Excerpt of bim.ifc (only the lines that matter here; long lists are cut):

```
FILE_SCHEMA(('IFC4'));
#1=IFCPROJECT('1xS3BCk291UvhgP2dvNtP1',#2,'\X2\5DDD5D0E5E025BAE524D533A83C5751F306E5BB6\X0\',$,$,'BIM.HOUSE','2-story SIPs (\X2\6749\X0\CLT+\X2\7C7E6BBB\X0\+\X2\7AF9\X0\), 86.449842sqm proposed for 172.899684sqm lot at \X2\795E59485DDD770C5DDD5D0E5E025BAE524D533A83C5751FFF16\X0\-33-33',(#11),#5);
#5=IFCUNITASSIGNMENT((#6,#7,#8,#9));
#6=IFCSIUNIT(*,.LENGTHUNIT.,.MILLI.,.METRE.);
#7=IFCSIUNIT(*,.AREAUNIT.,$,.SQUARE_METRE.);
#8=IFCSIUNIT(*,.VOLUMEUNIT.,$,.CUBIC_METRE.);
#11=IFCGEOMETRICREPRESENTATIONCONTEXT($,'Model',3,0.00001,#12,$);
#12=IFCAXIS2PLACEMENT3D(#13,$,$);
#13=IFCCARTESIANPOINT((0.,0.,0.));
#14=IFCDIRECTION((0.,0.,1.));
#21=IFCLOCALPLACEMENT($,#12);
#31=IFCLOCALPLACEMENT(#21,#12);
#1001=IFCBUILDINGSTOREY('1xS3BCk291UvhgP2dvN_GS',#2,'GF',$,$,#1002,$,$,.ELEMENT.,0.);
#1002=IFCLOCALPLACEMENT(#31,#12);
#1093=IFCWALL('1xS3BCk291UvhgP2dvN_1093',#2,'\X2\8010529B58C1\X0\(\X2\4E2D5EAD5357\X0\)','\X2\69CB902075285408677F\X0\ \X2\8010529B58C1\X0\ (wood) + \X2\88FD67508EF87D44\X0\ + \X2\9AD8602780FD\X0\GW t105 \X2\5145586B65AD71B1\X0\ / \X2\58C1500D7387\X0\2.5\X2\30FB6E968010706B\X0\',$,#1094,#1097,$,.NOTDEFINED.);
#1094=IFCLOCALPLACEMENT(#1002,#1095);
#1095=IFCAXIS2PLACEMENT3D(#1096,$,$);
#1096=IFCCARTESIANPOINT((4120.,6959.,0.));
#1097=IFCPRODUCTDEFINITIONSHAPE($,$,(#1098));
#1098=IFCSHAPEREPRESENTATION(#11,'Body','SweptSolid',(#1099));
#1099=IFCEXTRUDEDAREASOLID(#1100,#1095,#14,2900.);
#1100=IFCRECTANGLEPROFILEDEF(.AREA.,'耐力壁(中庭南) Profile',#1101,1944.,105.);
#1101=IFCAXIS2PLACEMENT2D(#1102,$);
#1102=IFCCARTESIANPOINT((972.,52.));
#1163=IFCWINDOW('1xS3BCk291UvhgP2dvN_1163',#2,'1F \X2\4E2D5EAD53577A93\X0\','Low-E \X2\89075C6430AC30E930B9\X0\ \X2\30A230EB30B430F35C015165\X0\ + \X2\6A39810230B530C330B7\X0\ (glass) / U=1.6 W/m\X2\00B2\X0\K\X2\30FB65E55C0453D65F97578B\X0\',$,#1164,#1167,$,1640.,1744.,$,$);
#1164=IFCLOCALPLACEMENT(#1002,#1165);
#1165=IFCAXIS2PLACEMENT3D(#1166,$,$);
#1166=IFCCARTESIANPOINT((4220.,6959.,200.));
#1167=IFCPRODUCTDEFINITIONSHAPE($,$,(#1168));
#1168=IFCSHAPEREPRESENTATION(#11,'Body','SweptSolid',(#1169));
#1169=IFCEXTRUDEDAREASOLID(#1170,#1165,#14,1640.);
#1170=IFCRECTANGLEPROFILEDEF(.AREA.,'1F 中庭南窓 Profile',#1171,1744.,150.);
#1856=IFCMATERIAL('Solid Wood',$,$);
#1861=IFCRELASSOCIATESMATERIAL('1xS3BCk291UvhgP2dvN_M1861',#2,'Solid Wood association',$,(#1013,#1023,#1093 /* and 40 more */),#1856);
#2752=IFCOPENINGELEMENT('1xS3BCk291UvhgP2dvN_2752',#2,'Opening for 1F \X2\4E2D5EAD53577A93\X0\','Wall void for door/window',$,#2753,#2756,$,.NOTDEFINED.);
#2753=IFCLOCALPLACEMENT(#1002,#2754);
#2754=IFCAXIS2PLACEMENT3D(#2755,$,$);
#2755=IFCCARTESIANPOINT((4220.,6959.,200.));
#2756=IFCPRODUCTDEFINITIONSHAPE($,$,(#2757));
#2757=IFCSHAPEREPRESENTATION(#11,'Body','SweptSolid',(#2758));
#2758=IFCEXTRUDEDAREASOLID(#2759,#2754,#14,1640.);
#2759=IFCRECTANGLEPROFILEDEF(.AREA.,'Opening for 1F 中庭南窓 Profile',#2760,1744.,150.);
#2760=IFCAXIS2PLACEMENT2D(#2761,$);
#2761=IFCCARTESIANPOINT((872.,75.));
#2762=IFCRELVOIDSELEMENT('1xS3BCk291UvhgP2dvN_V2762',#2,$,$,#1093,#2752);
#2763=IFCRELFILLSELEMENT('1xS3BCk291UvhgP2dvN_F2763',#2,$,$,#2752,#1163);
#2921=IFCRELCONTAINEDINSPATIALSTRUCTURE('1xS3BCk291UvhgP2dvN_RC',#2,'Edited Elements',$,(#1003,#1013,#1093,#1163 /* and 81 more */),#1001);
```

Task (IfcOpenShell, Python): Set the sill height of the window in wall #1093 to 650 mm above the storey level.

```python
import numpy as np
import ifcopenshell
import ifcopenshell.api.geometry
import ifcopenshell.geom
import ifcopenshell.util.element
import ifcopenshell.util.placement
import ifcopenshell.util.shape
import ifcopenshell.util.unit

model = ifcopenshell.open("bim.ifc")
unit_scale = ifcopenshell.util.unit.calculate_unit_scale(model)

window = model.by_guid("1xS3BCk291UvhgP2dvN_1163")
opening = window.FillsVoids[0].RelatingOpeningElement
storey = ifcopenshell.util.element.get_container(window, ifc_class="IfcBuildingStorey")
level = ifcopenshell.util.placement.get_local_placement(storey.ObjectPlacement)[2, 3]

# The opening's origin need not be at the sill, so measure its lowest point.
shape = ifcopenshell.geom.create_shape(ifcopenshell.geom.settings(), opening)
bottom = ifcopenshell.util.shape.get_shape_bottom_elevation(shape, shape.geometry) / unit_scale
dz = level + 650.0 - bottom

shift = np.array([0.0, 0.0, dz])
# The window is not placed relative to its opening, so move both.
for product in (opening, window):
    matrix = ifcopenshell.util.placement.get_local_placement(product.ObjectPlacement)
    matrix[:3, 3] += shift
    ifcopenshell.api.geometry.edit_object_placement(model, product=product, matrix=matrix, is_si=False)

print(f"moved by {dz * unit_scale:+.3f} m")

model.write("bim_edited.ifc")
```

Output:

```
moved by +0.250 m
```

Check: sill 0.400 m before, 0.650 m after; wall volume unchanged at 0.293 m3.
